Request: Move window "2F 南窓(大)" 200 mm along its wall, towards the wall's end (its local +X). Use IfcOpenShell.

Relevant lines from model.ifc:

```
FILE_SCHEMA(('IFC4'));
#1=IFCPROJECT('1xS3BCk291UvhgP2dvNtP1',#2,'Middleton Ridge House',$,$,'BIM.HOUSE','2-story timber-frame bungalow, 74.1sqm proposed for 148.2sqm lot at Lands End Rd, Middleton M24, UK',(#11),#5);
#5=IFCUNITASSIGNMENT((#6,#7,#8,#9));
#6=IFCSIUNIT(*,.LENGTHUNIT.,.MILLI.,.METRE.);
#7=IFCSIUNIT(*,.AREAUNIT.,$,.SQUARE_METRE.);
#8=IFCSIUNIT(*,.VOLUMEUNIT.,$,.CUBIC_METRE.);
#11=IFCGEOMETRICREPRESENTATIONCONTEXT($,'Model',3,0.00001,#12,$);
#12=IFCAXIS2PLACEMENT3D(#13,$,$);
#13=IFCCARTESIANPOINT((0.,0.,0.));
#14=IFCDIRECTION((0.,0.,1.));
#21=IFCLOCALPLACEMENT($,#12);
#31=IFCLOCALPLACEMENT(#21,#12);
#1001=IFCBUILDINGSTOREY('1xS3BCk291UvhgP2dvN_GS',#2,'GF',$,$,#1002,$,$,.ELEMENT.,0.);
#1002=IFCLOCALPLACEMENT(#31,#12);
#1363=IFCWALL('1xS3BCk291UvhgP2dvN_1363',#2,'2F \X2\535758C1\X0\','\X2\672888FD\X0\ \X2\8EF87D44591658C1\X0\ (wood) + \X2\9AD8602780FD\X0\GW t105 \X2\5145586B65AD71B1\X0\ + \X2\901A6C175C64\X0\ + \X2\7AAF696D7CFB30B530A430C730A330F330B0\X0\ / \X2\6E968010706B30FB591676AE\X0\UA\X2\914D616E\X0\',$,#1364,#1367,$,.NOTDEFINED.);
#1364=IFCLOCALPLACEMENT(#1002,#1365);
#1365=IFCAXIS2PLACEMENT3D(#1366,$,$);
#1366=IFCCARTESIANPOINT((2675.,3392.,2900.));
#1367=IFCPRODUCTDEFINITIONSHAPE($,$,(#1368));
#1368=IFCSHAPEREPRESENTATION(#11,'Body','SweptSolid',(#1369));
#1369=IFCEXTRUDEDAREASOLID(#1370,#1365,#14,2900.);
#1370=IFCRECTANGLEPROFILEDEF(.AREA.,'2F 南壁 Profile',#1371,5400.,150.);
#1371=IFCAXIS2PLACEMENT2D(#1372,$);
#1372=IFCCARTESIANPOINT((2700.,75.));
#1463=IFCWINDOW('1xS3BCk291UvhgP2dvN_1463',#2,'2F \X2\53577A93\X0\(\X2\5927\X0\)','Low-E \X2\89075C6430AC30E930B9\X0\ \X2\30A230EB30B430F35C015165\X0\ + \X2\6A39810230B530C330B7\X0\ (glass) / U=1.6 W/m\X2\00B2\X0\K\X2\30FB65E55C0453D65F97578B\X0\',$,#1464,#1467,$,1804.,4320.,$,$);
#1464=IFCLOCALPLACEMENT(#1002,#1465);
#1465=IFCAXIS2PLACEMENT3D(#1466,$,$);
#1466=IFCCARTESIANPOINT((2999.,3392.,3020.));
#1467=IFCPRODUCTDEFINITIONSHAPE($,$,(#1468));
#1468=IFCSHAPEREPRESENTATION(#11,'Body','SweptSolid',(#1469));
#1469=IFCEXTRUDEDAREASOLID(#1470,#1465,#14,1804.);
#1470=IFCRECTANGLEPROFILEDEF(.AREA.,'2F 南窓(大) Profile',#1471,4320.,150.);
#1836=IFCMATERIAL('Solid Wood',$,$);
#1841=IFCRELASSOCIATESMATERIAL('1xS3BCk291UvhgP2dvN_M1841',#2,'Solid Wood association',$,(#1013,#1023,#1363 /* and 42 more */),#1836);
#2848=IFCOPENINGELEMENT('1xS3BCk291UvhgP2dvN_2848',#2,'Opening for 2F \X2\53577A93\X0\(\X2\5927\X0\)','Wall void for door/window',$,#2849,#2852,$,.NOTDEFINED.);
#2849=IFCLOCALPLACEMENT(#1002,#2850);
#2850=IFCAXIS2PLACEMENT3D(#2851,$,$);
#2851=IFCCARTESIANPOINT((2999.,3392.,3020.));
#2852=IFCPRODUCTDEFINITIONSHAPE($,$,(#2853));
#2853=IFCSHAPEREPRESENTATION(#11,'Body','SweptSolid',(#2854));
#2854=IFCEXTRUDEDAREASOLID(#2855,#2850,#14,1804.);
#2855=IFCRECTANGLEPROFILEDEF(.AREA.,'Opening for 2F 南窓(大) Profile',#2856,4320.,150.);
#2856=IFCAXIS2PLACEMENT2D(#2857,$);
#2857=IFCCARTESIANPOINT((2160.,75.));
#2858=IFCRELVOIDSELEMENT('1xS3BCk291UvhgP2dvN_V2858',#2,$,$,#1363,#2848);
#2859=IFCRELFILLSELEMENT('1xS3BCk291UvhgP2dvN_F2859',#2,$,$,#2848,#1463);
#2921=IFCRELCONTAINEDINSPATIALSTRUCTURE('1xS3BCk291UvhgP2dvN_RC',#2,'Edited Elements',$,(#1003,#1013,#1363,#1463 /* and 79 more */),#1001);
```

```python
import ifcopenshell
import ifcopenshell.api.geometry
import ifcopenshell.util.placement
import ifcopenshell.util.unit

model = ifcopenshell.open("model.ifc")
unit_scale = ifcopenshell.util.unit.calculate_unit_scale(model)

window = model.by_id(1463)
opening = window.FillsVoids[0].RelatingOpeningElement
wall = opening.VoidsElements[0].RelatingBuildingElement

wall_matrix = ifcopenshell.util.placement.get_local_placement(wall.ObjectPlacement)
shift = wall_matrix[:3, 0] * 0.2 / unit_scale
before = ifcopenshell.util.placement.get_local_placement(window.ObjectPlacement)[:3, 3].copy()

# The window is not placed relative to its opening, so move both.
for product in (opening, window):
    matrix = ifcopenshell.util.placement.get_local_placement(product.ObjectPlacement)
    matrix[:3, 3] += shift
    ifcopenshell.api.geometry.edit_object_placement(model, product=product, matrix=matrix, is_si=False)

after = ifcopenshell.util.placement.get_local_placement(window.ObjectPlacement)[:3, 3]
print("window moved by", (after - before).round(3) + 0.0)

model.write("model_edited.ifc")
```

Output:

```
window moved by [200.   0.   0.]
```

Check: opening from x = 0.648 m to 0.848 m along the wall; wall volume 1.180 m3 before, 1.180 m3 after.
